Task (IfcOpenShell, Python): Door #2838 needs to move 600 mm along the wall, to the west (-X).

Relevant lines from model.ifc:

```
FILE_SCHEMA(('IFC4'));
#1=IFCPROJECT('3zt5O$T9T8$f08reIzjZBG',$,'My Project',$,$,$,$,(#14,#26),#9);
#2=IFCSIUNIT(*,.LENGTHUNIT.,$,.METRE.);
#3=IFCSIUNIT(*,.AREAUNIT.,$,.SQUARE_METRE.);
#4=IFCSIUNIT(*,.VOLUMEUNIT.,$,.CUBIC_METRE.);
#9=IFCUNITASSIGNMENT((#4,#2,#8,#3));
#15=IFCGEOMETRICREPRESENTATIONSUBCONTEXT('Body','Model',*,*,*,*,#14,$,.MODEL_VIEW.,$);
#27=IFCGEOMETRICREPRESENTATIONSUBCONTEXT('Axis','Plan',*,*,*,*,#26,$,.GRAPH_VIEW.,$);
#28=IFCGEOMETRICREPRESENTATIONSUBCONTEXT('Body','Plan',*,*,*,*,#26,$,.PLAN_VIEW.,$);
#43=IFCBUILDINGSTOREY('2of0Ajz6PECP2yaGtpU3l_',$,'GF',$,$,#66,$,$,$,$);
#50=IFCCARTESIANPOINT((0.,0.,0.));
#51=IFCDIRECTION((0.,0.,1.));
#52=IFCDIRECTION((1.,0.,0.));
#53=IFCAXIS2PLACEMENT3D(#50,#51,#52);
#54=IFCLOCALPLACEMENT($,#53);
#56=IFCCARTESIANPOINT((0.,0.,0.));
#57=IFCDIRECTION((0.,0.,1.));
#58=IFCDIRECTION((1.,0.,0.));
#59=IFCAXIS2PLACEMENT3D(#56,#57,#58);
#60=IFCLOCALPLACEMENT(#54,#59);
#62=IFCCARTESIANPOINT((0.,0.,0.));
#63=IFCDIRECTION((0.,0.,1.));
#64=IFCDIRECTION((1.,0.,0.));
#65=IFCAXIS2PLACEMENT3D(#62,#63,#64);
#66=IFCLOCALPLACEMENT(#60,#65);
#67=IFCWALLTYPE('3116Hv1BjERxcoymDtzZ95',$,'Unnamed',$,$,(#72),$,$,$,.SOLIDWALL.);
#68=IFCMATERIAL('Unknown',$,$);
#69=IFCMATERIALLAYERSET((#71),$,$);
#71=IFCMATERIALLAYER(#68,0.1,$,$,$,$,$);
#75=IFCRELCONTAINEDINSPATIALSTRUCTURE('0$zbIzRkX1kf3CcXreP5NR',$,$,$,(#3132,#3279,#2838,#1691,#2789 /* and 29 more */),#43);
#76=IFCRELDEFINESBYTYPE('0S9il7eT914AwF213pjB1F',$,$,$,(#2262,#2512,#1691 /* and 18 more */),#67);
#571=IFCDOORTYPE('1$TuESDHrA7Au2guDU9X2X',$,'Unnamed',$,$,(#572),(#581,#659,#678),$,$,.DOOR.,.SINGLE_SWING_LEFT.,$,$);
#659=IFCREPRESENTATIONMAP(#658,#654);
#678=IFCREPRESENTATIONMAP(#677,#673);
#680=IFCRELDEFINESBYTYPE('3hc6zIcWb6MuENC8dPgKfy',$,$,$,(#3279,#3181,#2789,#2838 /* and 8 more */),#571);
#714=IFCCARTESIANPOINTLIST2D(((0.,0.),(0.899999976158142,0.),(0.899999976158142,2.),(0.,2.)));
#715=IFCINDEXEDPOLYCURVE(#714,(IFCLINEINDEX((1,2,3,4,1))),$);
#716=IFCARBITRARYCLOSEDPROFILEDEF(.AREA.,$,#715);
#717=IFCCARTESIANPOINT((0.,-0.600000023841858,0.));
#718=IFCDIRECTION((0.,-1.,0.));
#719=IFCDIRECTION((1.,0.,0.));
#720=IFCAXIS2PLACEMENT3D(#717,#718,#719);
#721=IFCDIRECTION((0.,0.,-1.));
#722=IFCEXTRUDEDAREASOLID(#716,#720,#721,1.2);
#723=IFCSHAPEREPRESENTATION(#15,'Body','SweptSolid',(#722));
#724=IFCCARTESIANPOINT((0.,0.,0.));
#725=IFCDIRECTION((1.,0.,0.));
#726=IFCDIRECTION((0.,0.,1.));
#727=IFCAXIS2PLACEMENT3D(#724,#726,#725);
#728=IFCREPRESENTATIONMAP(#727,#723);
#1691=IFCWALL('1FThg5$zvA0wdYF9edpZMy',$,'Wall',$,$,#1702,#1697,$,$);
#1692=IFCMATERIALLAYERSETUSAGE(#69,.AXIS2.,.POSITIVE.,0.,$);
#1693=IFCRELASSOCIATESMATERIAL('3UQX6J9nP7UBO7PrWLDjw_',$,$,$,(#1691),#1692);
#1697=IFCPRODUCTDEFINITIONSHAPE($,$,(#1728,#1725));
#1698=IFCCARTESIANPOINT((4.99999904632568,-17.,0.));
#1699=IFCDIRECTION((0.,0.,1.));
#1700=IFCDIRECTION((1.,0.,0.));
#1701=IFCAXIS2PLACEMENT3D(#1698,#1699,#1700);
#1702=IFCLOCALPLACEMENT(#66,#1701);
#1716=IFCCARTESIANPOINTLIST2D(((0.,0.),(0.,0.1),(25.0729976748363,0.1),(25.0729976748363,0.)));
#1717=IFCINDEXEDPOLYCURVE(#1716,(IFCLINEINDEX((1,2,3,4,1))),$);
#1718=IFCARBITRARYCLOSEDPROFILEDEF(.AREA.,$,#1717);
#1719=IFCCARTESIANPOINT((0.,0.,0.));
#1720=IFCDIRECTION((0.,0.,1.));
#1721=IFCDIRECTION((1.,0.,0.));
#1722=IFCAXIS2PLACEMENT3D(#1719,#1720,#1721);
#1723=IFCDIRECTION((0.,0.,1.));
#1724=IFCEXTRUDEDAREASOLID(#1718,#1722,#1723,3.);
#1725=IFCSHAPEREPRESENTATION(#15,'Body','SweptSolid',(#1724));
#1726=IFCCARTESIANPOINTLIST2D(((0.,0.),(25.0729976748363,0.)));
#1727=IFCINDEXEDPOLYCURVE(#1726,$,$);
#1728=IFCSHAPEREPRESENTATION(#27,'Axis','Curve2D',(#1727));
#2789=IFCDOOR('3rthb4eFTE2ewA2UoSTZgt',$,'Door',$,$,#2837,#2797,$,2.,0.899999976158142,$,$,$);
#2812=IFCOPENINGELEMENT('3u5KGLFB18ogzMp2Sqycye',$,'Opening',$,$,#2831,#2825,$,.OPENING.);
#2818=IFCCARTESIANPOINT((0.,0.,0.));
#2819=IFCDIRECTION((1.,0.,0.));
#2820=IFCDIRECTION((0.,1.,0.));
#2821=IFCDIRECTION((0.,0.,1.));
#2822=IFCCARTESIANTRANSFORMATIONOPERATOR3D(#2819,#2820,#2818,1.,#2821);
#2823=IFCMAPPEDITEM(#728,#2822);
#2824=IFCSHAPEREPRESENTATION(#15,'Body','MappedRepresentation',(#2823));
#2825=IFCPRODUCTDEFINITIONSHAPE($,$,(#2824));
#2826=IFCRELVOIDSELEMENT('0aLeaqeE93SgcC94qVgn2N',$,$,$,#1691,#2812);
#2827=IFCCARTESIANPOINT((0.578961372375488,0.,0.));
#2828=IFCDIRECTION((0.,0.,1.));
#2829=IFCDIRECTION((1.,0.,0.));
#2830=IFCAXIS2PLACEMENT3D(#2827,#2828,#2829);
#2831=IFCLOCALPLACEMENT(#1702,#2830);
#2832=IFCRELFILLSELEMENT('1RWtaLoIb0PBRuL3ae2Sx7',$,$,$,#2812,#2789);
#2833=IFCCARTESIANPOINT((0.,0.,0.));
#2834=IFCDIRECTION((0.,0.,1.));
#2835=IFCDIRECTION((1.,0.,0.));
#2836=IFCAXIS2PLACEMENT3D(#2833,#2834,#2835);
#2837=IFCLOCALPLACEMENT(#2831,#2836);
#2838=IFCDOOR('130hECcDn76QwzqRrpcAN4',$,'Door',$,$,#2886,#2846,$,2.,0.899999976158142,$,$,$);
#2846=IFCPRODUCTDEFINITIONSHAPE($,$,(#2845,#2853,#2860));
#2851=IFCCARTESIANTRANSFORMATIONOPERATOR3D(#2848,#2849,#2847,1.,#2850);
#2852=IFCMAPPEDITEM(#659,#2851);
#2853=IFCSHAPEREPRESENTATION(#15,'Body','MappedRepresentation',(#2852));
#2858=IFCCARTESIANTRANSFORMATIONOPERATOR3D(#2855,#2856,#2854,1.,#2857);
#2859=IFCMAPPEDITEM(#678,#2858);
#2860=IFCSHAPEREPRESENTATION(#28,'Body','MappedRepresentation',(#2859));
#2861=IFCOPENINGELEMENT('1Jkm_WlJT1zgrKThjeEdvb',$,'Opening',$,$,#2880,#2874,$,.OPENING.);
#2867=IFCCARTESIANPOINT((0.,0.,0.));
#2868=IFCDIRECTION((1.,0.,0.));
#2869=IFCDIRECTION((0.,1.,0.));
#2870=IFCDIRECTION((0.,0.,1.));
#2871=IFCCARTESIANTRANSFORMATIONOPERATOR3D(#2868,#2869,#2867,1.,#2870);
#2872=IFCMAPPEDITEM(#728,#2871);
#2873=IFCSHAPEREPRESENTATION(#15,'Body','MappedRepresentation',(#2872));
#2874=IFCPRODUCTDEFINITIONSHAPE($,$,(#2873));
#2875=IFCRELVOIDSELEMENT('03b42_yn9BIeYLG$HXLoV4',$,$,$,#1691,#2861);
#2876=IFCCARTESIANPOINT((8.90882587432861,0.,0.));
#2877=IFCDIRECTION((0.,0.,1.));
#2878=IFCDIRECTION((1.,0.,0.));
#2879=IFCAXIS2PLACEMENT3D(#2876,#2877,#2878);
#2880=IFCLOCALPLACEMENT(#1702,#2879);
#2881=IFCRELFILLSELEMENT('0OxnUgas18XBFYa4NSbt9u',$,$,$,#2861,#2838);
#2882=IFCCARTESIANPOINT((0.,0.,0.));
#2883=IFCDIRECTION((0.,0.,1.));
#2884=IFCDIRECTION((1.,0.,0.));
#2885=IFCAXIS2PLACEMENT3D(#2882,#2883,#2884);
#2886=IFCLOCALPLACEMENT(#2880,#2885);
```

```python
import ifcopenshell
import ifcopenshell.api.geometry
import ifcopenshell.util.placement

model = ifcopenshell.open("model.ifc")

door = model.by_guid("130hECcDn76QwzqRrpcAN4")
opening = door.FillsVoids[0].RelatingOpeningElement
wall = opening.VoidsElements[0].RelatingBuildingElement

wall_matrix = ifcopenshell.util.placement.get_local_placement(wall.ObjectPlacement)
shift = wall_matrix[:3, 0] * -0.6
before = ifcopenshell.util.placement.get_local_placement(door.ObjectPlacement)[:3, 3].copy()

# The door is placed relative to its opening, so it follows when the opening moves.
matrix = ifcopenshell.util.placement.get_local_placement(opening.ObjectPlacement)
matrix[:3, 3] += shift
ifcopenshell.api.geometry.edit_object_placement(
    model, product=opening, matrix=matrix, is_si=False, should_transform_children=True
)

after = ifcopenshell.util.placement.get_local_placement(door.ObjectPlacement)[:3, 3]
print("door moved by", (after - before).round(3) + 0.0)

model.write("model_rev.ifc")
```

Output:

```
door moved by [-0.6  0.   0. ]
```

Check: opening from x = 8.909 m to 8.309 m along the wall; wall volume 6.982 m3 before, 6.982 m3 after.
